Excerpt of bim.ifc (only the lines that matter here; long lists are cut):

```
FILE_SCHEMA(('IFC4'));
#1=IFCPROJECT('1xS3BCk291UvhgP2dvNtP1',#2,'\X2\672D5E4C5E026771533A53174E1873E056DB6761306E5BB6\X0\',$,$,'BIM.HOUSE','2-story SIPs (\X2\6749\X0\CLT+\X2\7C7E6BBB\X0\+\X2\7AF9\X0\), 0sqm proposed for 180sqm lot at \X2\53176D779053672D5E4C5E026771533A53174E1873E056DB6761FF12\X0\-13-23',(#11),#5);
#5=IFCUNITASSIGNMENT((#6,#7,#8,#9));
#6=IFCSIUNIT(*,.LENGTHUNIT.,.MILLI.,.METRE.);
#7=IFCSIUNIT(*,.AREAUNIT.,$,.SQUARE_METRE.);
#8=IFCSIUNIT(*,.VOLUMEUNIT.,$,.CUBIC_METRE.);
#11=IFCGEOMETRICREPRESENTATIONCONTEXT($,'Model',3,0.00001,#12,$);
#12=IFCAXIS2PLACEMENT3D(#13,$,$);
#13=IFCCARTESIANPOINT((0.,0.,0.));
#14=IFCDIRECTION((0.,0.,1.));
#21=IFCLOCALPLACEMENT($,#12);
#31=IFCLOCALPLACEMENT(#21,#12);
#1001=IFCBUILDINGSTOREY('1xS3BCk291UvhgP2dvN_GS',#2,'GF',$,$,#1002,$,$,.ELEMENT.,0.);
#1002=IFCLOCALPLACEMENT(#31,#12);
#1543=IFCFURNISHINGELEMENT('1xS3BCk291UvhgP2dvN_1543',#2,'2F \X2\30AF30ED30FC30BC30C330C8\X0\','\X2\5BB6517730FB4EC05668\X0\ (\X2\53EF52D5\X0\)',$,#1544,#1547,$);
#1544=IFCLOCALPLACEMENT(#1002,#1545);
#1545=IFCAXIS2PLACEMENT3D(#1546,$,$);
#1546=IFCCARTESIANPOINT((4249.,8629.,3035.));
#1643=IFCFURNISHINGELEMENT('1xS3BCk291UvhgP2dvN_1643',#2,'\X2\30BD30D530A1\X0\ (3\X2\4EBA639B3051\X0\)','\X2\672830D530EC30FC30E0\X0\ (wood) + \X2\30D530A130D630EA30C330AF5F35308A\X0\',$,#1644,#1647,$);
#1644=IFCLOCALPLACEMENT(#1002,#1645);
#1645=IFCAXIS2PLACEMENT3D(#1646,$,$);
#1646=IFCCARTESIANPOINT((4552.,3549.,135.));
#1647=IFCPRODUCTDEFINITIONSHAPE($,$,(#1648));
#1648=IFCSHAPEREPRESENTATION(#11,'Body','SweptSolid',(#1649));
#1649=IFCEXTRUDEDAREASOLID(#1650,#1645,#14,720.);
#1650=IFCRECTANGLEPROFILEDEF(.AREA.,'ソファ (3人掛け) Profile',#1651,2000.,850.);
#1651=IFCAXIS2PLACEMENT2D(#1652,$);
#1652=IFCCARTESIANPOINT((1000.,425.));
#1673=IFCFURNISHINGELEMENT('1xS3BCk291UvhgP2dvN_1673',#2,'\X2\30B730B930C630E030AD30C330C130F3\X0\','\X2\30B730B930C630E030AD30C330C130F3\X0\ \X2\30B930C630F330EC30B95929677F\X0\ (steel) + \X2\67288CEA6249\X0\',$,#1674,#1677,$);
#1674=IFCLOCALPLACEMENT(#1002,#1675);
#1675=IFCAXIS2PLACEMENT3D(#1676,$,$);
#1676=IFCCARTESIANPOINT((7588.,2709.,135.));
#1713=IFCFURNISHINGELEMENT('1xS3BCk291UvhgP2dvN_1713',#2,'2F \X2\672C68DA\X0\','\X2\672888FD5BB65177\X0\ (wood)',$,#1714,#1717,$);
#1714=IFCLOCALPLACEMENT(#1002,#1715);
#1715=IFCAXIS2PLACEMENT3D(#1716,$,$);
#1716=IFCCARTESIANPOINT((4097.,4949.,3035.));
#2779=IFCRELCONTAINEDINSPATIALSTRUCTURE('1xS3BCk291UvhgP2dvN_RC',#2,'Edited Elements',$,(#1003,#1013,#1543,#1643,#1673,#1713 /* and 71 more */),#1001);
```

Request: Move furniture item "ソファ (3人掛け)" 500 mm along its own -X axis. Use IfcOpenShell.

```python
import ifcopenshell
import ifcopenshell.api.geometry
import ifcopenshell.util.placement
import ifcopenshell.util.unit

model = ifcopenshell.open("bim.ifc")
unit_scale = ifcopenshell.util.unit.calculate_unit_scale(model)

item = model.by_id(1643)
matrix = ifcopenshell.util.placement.get_local_placement(item.ObjectPlacement)
matrix[:3, 3] -= matrix[:3, 0] * 0.5 / unit_scale
ifcopenshell.api.geometry.edit_object_placement(model, product=item, matrix=matrix, is_si=False)

print(ifcopenshell.util.placement.get_local_placement(item.ObjectPlacement).round(3) + 0.0)

model.write("bim_updated.ifc")
```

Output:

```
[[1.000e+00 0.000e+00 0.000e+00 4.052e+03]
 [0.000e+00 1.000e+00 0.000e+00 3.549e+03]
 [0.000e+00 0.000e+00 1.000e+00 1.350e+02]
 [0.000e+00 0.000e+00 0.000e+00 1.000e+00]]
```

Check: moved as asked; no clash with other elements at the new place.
